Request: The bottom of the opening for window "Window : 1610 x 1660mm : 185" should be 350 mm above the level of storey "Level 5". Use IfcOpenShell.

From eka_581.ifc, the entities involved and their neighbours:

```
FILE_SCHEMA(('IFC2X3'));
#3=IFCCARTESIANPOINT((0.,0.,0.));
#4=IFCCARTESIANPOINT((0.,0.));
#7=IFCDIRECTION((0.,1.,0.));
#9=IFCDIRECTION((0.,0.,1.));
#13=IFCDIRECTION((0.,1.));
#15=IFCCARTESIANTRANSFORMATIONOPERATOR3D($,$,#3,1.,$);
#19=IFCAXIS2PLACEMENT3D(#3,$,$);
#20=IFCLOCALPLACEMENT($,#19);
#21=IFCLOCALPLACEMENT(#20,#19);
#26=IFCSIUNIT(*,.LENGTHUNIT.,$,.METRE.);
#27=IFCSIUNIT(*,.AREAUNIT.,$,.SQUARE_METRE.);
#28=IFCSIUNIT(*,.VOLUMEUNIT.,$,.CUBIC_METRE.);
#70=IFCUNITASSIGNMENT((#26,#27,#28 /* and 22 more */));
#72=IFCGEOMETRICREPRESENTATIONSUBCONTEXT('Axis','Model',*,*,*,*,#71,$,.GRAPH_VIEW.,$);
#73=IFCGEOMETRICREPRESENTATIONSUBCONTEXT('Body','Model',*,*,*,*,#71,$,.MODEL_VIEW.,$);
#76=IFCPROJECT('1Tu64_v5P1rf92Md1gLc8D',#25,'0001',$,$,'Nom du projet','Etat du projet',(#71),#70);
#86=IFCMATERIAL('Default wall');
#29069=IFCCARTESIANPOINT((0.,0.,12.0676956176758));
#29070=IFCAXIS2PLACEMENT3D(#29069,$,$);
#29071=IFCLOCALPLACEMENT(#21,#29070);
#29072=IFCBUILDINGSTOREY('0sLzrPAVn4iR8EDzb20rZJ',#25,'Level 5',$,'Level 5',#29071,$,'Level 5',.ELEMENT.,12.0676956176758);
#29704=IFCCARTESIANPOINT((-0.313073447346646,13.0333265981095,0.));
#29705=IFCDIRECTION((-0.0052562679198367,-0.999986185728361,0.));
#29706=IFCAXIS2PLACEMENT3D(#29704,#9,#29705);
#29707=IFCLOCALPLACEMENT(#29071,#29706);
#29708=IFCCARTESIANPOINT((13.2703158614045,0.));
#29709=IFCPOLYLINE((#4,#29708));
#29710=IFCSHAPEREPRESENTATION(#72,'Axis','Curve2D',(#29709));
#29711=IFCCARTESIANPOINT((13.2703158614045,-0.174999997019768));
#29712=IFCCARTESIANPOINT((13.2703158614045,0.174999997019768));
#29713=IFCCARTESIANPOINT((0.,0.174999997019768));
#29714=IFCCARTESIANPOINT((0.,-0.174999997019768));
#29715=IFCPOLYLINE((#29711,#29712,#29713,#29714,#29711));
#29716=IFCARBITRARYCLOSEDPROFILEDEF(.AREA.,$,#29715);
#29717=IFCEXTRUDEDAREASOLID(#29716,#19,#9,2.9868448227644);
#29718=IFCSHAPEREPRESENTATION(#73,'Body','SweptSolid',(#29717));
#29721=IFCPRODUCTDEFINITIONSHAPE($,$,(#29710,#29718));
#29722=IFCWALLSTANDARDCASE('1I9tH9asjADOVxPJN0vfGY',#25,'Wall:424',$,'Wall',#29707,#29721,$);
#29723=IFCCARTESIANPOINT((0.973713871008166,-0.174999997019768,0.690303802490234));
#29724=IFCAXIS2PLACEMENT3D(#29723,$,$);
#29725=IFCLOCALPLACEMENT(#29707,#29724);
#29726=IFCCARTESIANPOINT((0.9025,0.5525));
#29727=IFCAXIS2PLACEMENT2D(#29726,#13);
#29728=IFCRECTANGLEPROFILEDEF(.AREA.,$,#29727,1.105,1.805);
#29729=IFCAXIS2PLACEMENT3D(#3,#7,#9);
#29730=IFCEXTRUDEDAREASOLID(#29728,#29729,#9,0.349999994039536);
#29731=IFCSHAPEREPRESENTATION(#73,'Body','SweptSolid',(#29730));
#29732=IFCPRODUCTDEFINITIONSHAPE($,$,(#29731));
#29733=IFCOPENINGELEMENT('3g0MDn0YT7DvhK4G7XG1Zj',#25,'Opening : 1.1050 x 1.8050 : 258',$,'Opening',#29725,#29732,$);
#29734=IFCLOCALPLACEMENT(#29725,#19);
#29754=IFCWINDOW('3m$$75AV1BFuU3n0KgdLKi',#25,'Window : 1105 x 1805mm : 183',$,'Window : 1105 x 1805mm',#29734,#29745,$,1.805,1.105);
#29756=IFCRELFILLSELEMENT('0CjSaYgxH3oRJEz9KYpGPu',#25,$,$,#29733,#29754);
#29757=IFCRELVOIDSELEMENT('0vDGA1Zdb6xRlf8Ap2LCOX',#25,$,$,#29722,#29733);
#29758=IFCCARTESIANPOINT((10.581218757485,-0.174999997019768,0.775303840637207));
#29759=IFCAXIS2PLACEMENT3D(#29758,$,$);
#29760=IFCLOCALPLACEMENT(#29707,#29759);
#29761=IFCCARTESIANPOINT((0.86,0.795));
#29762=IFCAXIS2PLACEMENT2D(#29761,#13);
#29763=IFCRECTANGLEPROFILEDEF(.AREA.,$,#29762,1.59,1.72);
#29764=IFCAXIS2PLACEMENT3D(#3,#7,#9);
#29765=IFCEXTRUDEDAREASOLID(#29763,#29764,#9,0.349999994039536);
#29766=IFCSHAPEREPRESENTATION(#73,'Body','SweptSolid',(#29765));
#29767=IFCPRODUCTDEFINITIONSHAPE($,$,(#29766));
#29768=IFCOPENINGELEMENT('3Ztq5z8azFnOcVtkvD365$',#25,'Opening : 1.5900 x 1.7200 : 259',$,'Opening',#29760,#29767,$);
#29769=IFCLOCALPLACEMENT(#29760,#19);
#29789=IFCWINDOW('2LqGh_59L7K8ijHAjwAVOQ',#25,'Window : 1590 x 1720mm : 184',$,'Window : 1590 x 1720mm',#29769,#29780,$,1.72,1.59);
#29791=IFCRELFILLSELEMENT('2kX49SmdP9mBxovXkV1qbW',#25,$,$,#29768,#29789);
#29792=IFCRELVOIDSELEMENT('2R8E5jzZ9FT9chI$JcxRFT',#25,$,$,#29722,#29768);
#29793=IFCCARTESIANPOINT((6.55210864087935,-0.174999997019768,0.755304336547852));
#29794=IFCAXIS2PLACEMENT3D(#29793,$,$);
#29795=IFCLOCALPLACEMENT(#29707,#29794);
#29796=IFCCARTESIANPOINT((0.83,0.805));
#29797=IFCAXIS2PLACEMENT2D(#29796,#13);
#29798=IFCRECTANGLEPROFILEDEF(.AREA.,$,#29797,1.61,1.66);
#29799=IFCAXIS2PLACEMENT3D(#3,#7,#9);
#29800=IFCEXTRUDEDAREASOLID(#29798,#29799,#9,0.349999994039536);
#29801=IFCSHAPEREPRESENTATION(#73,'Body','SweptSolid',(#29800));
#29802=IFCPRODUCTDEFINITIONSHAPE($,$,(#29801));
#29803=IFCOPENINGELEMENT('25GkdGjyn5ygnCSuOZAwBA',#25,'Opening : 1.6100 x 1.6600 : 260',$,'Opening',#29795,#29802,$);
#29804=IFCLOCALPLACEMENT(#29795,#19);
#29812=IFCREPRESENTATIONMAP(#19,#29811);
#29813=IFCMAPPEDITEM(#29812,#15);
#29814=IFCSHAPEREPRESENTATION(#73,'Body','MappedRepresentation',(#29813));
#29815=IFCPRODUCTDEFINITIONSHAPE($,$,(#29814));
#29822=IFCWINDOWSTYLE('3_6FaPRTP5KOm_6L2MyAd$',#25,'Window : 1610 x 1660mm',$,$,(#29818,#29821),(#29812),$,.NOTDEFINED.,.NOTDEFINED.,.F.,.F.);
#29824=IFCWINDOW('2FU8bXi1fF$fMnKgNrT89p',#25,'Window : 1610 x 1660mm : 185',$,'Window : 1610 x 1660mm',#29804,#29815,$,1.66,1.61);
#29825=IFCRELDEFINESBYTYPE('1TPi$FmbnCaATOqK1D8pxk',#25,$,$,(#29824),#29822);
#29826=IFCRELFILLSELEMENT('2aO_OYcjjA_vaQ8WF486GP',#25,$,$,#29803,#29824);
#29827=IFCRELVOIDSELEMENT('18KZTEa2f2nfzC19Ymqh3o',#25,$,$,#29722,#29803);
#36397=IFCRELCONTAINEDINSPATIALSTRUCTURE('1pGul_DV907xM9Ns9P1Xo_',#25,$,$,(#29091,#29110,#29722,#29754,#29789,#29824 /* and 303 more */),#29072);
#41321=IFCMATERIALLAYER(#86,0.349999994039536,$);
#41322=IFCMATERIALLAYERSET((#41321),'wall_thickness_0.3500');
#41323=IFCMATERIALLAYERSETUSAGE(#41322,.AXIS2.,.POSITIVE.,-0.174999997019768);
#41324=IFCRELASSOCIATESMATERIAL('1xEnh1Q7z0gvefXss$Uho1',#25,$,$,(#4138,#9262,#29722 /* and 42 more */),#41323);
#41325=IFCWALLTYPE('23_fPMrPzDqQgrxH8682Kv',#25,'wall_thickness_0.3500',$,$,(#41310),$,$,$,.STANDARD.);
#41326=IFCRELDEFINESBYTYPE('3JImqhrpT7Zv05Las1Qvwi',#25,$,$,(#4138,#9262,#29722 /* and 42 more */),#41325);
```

```python
import numpy as np
import ifcopenshell
import ifcopenshell.api.geometry
import ifcopenshell.geom
import ifcopenshell.util.element
import ifcopenshell.util.placement
import ifcopenshell.util.shape
import ifcopenshell.util.unit

model = ifcopenshell.open("eka_581.ifc")
unit_scale = ifcopenshell.util.unit.calculate_unit_scale(model)

window = model.by_guid("2FU8bXi1fF$fMnKgNrT89p")
opening = window.FillsVoids[0].RelatingOpeningElement
storey = ifcopenshell.util.element.get_container(window, ifc_class="IfcBuildingStorey")
level = ifcopenshell.util.placement.get_local_placement(storey.ObjectPlacement)[2, 3]

# The opening's origin need not be at the sill, so measure its lowest point.
shape = ifcopenshell.geom.create_shape(ifcopenshell.geom.settings(), opening)
bottom = ifcopenshell.util.shape.get_shape_bottom_elevation(shape, shape.geometry) / unit_scale
dz = level + 0.35 - bottom

shift = np.array([0.0, 0.0, dz])
# The window is placed relative to its opening, so it follows when the opening moves.
matrix = ifcopenshell.util.placement.get_local_placement(opening.ObjectPlacement)
matrix[:3, 3] += shift
ifcopenshell.api.geometry.edit_object_placement(
    model, product=opening, matrix=matrix, is_si=False, should_transform_children=True
)

print(f"moved by {dz * unit_scale:+.3f} m")

model.write("eka_581_updated.ifc")
```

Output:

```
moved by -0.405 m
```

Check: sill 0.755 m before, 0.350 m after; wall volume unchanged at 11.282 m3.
